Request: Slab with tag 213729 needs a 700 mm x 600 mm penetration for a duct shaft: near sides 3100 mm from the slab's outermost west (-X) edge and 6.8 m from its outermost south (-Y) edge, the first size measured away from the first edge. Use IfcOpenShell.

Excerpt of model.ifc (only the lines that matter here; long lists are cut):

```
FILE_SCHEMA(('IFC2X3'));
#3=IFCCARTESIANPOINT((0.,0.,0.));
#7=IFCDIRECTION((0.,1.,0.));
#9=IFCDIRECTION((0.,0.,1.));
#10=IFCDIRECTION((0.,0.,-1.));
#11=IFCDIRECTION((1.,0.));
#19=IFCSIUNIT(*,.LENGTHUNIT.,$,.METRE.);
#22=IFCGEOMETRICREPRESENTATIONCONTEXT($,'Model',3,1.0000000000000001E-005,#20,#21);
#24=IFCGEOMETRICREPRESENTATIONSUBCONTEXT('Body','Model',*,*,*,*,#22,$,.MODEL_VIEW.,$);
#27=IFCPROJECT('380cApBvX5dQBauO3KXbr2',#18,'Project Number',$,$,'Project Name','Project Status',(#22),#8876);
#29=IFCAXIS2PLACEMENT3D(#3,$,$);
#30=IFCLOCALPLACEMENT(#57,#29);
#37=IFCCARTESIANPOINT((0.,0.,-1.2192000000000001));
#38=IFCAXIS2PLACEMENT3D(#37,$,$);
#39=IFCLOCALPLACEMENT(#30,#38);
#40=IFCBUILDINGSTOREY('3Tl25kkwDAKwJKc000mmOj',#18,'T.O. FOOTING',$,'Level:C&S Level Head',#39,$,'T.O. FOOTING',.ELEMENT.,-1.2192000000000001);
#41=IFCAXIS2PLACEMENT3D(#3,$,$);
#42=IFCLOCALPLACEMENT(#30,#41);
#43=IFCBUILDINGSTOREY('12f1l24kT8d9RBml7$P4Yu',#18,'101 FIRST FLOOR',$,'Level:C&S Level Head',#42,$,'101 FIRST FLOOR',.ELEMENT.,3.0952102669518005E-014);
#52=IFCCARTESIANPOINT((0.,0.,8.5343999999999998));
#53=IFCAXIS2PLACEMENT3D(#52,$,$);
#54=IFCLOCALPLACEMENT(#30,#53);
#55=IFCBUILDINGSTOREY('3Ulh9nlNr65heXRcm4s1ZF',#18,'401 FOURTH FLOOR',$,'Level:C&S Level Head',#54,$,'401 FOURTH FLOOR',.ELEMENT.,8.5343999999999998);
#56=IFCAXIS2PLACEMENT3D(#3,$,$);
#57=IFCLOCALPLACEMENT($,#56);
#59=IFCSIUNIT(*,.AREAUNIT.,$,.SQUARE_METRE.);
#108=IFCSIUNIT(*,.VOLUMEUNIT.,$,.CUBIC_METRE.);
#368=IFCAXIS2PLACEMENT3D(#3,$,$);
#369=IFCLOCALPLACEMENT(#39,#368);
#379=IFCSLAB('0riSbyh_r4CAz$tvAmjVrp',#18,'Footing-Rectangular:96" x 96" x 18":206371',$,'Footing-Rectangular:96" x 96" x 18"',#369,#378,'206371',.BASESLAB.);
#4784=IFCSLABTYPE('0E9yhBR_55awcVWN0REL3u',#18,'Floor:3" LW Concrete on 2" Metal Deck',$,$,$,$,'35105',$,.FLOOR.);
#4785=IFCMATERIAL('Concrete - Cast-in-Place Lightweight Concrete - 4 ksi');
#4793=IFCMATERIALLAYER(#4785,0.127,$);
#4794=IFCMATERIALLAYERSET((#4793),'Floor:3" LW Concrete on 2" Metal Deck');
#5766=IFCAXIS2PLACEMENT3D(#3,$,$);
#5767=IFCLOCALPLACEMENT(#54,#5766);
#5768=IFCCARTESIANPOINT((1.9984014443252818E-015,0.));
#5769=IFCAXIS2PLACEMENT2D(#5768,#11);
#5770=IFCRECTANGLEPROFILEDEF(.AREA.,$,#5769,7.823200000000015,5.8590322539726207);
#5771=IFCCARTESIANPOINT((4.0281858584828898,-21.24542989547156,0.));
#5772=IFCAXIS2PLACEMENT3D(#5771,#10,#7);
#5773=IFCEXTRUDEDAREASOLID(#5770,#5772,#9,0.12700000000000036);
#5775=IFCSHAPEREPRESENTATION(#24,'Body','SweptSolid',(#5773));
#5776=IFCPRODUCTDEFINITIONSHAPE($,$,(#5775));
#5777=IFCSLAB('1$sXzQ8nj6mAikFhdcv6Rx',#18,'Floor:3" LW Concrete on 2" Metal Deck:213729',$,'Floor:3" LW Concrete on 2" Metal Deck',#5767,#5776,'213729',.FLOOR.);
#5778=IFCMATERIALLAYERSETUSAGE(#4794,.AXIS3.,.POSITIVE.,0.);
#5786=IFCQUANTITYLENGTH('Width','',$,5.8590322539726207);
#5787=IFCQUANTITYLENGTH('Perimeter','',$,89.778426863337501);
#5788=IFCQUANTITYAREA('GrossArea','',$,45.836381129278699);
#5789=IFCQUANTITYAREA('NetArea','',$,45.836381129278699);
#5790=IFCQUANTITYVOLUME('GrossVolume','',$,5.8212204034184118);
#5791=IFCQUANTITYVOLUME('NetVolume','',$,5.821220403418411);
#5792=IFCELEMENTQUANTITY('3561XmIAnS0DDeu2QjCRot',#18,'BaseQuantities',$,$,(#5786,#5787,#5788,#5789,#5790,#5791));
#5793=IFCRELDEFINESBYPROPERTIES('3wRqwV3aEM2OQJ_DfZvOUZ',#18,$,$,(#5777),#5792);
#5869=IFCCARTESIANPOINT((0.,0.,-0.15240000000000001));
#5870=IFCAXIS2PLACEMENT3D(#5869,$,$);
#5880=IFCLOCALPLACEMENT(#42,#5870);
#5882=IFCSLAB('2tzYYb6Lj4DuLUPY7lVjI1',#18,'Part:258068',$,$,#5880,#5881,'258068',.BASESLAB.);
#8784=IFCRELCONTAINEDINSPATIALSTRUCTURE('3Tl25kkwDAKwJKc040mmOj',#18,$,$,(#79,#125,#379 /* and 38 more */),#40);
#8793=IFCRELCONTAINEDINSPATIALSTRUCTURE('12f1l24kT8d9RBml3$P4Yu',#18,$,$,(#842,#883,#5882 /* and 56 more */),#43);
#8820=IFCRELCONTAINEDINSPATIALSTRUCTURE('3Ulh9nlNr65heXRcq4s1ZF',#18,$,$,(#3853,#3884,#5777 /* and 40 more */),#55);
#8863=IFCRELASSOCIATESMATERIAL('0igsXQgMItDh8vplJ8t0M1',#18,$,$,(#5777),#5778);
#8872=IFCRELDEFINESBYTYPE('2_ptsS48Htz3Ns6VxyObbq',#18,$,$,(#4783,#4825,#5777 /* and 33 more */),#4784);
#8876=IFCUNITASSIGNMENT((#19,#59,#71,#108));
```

```python
import numpy as np
import ifcopenshell
import ifcopenshell.api.feature
import ifcopenshell.api.geometry
import ifcopenshell.api.pset
import ifcopenshell.api.root
import ifcopenshell.geom
import ifcopenshell.util.element
import ifcopenshell.util.placement
import ifcopenshell.util.representation
import ifcopenshell.util.shape
import ifcopenshell.util.unit

model = ifcopenshell.open("model.ifc")
unit_scale = ifcopenshell.util.unit.calculate_unit_scale(model)
area_scale = ifcopenshell.util.unit.calculate_unit_scale(model, "AREAUNIT")
volume_scale = ifcopenshell.util.unit.calculate_unit_scale(model, "VOLUMEUNIT")
settings = ifcopenshell.geom.settings()


def volume(element):
    """Net volume in cubic metres, openings subtracted."""
    shape = ifcopenshell.geom.create_shape(settings, element)
    return ifcopenshell.util.shape.get_volume(shape.geometry)


slab = model.by_guid("1$sXzQ8nj6mAikFhdcv6Rx")
before = volume(slab)

# Extent in the slab's own axes, in metres. The edges named are its -X and -Y sides.
slab_shape = ifcopenshell.geom.create_shape(settings, slab)
vertices = ifcopenshell.util.shape.get_vertices(slab_shape.geometry)
x_min, y_min, bottom = vertices.min(axis=0)
top = vertices[:, 2].max()

opening = ifcopenshell.api.root.create_entity(model, ifc_class="IfcOpeningElement", name="Duct shaft opening")
context = ifcopenshell.util.representation.get_context(model, "Model", "Body", "MODEL_VIEW")
width, depth = 0.7, 0.6
outline = [(0.0, 0.0), (width, 0.0), (width, depth), (0.0, depth), (0.0, 0.0)]
# Overshoot both faces by 50 mm so the cut is clean.
shape = ifcopenshell.api.geometry.add_slab_representation(
    model, context=context, depth=top - bottom + 0.1, polyline=outline
)
ifcopenshell.api.geometry.assign_representation(model, product=opening, representation=shape)

matrix = ifcopenshell.util.placement.get_local_placement(slab.ObjectPlacement)
matrix[:, 3] = matrix @ np.append(np.array([x_min + 3.1, y_min + 6.8, bottom - 0.05]) / unit_scale, 1.0)
ifcopenshell.api.geometry.edit_object_placement(model, product=opening, matrix=matrix, is_si=False)
ifcopenshell.api.feature.add_feature(model, feature=opening, element=slab)

after = volume(slab)

# Update the slab's stored quantities.
qto = model.by_id(ifcopenshell.util.element.get_pset(slab, "BaseQuantities", should_inherit=False)["id"])
ifcopenshell.api.pset.edit_qto(model, qto=qto, properties={
    "NetArea": after / (top - bottom) / area_scale,
    "NetVolume": after / volume_scale,
})

print(f"slab volume {before:.3f} -> {after:.3f} m3")

model.write("model_edited.ifc")
```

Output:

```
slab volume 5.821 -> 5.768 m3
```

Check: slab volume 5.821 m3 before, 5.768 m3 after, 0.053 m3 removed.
